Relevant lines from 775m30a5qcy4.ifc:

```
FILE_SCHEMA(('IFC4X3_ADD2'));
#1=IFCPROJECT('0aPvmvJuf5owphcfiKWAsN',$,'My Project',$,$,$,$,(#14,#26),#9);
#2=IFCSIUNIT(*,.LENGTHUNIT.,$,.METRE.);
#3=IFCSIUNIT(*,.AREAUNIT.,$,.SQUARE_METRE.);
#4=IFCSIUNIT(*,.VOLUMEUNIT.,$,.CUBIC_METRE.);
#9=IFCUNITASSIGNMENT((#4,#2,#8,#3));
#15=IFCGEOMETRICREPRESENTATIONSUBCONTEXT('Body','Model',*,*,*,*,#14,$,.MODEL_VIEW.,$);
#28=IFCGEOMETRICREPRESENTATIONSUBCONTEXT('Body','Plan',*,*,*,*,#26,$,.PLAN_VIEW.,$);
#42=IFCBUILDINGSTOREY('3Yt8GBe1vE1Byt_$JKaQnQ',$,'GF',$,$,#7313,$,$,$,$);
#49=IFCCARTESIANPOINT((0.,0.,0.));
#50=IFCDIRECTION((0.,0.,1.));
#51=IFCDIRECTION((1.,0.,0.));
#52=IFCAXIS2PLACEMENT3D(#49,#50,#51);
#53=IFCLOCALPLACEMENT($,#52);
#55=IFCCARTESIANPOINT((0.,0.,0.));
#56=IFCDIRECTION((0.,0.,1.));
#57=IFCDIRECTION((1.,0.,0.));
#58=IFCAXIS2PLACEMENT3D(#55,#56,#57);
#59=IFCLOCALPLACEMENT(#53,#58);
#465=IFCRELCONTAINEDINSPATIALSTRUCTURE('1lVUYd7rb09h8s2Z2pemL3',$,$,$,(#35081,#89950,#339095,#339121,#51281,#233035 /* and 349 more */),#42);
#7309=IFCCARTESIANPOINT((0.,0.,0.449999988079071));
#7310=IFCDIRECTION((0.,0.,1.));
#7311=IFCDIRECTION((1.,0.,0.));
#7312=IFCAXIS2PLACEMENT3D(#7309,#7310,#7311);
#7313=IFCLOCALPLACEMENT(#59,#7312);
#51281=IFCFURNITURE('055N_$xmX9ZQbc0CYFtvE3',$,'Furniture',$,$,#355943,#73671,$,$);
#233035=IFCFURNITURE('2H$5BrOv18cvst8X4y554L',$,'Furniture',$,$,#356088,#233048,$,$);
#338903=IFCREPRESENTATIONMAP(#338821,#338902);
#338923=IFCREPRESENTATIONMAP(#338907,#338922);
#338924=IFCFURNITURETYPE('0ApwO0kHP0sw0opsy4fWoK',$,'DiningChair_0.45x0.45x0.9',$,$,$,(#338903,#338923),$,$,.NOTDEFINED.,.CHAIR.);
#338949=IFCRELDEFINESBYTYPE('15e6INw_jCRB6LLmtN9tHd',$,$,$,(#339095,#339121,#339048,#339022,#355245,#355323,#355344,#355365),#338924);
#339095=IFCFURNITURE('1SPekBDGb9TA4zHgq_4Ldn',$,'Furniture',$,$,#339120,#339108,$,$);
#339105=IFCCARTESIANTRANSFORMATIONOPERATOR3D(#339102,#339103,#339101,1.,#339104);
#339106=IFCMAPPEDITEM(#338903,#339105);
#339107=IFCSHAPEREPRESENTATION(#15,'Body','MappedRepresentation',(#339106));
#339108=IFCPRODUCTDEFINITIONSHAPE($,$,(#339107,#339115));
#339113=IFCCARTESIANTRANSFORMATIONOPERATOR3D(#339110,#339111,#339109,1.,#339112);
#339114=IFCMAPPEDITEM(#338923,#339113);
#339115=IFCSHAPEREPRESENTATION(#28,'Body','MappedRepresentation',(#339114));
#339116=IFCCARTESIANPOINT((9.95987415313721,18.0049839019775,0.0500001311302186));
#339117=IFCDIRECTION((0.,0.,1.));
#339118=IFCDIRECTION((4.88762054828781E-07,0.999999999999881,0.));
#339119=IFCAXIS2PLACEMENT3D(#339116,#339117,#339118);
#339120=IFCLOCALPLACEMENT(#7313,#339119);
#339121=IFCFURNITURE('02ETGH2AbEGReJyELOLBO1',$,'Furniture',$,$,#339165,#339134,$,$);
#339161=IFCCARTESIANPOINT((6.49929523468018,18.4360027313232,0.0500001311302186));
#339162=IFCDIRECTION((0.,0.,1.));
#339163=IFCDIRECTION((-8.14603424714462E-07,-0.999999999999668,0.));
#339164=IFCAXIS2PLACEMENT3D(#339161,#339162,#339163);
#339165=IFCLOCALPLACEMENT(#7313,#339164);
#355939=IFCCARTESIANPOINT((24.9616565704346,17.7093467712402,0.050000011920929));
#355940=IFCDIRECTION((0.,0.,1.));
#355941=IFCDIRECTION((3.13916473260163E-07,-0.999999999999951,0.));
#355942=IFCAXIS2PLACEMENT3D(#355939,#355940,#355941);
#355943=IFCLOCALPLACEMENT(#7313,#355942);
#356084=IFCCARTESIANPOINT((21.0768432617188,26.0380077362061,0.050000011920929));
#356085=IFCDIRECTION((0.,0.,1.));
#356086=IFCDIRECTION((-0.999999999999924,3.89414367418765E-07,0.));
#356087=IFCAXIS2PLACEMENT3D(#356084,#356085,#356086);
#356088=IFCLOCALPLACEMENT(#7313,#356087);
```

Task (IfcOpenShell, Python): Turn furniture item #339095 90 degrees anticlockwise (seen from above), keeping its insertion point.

```python
import ifcopenshell
import ifcopenshell.api.geometry
import ifcopenshell.util.placement

model = ifcopenshell.open("775m30a5qcy4.ifc")

item = model.by_id(339095)
matrix = ifcopenshell.util.placement.get_local_placement(item.ObjectPlacement)
matrix = matrix @ ifcopenshell.util.placement.rotation(90, "Z")
ifcopenshell.api.geometry.edit_object_placement(model, product=item, matrix=matrix, is_si=False)

print(ifcopenshell.util.placement.get_local_placement(item.ObjectPlacement).round(3) + 0.0)

model.write("775m30a5qcy4_edited.ifc")
```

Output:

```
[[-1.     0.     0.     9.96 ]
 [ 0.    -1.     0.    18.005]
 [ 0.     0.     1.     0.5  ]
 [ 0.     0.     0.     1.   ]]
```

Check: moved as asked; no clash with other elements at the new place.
